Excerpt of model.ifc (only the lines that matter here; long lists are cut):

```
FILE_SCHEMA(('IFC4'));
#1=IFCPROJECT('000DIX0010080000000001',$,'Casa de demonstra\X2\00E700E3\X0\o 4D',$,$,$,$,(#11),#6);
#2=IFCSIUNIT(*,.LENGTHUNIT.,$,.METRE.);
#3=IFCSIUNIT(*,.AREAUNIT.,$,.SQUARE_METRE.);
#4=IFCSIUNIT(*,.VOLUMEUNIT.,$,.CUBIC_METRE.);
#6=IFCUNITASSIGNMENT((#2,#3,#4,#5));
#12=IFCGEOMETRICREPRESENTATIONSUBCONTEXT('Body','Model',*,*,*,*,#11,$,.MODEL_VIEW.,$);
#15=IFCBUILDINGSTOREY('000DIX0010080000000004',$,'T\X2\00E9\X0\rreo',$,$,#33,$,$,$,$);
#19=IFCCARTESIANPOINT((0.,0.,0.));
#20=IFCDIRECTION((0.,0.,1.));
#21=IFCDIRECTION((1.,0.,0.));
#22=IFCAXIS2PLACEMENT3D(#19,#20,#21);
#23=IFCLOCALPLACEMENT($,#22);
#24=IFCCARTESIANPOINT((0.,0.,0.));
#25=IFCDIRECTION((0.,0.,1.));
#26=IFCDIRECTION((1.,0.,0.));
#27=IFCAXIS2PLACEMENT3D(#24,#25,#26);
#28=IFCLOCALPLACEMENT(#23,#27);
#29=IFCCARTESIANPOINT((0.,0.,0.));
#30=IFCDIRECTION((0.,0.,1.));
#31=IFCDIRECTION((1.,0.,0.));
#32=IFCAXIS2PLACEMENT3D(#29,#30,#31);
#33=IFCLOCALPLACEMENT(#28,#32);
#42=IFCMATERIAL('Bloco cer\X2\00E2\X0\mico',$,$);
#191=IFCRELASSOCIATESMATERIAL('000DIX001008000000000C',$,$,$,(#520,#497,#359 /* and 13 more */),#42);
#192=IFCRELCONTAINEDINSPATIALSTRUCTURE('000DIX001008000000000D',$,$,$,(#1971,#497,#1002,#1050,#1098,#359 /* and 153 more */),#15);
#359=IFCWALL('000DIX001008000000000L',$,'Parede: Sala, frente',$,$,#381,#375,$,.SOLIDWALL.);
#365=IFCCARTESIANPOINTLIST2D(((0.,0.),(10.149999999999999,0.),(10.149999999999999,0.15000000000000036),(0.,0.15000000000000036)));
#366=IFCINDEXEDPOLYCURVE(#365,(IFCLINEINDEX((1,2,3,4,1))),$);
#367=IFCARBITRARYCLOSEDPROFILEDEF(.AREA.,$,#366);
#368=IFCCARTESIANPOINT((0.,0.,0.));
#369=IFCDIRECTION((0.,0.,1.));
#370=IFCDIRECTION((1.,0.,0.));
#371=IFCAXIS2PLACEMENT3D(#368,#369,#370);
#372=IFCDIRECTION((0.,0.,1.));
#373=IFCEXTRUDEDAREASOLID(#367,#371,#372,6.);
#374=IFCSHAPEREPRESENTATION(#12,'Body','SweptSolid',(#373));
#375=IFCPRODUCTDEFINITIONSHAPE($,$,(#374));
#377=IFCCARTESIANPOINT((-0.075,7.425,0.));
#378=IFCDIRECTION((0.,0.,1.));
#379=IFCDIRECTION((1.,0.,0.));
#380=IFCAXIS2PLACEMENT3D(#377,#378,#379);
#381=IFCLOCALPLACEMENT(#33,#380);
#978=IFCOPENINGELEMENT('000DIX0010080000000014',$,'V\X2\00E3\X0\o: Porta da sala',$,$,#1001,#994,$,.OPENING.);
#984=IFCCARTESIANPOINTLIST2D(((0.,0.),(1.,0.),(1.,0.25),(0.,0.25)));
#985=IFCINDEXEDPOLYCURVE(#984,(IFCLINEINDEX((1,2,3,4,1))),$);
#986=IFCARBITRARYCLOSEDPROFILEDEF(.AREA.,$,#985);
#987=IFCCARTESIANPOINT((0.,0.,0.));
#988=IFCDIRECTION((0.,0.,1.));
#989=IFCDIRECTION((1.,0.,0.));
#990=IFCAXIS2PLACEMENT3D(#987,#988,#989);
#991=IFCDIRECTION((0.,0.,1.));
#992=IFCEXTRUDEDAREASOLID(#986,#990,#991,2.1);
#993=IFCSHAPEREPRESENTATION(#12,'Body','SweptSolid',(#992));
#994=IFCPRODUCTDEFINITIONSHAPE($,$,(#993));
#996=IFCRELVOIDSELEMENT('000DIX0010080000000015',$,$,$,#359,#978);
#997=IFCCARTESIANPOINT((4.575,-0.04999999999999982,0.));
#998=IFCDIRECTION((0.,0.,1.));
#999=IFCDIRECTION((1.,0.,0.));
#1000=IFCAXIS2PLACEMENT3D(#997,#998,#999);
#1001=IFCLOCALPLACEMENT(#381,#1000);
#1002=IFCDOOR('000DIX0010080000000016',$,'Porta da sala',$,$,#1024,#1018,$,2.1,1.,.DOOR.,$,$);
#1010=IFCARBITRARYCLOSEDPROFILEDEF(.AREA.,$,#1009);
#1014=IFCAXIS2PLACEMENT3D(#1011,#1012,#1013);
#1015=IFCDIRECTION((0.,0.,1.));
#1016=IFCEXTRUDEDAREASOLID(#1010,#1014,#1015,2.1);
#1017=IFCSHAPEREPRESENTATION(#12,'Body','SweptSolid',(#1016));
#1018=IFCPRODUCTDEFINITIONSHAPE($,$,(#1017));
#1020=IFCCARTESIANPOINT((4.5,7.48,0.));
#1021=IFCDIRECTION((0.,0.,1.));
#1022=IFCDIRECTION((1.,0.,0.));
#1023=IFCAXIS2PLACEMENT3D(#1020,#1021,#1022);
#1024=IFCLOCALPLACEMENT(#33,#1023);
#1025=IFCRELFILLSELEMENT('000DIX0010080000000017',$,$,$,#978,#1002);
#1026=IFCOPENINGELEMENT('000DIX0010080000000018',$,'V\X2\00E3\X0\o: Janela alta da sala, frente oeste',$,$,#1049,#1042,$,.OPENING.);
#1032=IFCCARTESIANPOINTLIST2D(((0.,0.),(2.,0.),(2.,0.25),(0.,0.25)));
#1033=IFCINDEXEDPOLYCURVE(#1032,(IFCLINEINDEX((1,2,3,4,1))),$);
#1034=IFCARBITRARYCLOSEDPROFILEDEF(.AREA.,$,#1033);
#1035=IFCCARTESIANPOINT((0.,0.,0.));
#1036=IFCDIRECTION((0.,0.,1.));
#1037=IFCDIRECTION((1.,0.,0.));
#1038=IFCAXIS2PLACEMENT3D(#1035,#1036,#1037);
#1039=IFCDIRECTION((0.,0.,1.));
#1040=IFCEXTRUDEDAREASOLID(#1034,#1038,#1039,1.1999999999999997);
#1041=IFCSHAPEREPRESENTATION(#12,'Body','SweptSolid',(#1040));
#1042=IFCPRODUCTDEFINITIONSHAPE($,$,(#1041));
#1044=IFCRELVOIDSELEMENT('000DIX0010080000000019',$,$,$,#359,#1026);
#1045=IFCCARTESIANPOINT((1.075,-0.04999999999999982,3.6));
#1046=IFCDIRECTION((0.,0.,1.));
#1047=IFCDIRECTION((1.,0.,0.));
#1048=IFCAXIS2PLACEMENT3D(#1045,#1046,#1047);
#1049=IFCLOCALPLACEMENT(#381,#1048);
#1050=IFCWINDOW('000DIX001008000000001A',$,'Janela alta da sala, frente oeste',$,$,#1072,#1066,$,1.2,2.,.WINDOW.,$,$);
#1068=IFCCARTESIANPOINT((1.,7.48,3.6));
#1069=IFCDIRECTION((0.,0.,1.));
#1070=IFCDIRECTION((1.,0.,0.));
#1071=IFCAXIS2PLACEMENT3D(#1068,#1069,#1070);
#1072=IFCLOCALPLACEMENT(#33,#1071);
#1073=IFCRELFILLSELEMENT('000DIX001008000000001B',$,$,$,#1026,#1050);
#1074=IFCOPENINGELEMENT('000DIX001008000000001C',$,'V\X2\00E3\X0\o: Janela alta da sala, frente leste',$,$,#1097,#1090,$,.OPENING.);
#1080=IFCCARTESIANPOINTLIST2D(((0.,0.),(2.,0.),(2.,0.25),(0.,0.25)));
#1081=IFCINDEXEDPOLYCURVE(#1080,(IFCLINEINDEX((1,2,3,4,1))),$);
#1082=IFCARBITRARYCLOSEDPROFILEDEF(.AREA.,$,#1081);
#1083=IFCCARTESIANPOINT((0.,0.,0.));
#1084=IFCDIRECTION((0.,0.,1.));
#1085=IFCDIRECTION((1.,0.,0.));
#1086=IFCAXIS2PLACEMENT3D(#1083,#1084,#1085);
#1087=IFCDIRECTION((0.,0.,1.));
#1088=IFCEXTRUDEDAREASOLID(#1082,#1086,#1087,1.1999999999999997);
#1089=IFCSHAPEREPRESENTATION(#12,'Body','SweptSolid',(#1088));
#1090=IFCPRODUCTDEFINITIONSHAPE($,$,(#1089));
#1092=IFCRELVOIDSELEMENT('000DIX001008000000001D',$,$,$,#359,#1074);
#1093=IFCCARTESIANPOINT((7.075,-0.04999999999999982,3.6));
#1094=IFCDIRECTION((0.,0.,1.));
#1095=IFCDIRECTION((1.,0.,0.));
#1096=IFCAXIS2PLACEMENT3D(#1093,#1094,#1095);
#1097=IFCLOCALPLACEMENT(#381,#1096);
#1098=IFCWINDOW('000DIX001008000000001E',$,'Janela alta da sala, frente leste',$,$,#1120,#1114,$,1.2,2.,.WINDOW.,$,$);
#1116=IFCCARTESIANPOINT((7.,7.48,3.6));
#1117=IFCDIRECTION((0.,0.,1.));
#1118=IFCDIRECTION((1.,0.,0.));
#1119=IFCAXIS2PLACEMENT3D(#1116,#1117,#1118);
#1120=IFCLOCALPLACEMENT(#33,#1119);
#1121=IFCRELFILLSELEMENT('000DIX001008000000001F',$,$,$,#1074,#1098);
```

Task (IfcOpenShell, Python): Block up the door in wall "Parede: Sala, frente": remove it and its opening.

```python
import ifcopenshell
import ifcopenshell.api.feature
import ifcopenshell.api.root
import ifcopenshell.geom
import ifcopenshell.util.shape

model = ifcopenshell.open("model.ifc")
settings = ifcopenshell.geom.settings()


def volume(element):
    """Net volume in cubic metres, openings subtracted."""
    shape = ifcopenshell.geom.create_shape(settings, element)
    return ifcopenshell.util.shape.get_volume(shape.geometry)


door = model.by_guid("000DIX0010080000000016")
opening = door.FillsVoids[0].RelatingOpeningElement
wall = opening.VoidsElements[0].RelatingBuildingElement
before = volume(wall)

ifcopenshell.api.root.remove_product(model, product=door)
ifcopenshell.api.feature.remove_feature(model, feature=opening)

after = volume(wall)

print(f"wall volume {before:.3f} -> {after:.3f} m3")

model.write("model_updated.ifc")
```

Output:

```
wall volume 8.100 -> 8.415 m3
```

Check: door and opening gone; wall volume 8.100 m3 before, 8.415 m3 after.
